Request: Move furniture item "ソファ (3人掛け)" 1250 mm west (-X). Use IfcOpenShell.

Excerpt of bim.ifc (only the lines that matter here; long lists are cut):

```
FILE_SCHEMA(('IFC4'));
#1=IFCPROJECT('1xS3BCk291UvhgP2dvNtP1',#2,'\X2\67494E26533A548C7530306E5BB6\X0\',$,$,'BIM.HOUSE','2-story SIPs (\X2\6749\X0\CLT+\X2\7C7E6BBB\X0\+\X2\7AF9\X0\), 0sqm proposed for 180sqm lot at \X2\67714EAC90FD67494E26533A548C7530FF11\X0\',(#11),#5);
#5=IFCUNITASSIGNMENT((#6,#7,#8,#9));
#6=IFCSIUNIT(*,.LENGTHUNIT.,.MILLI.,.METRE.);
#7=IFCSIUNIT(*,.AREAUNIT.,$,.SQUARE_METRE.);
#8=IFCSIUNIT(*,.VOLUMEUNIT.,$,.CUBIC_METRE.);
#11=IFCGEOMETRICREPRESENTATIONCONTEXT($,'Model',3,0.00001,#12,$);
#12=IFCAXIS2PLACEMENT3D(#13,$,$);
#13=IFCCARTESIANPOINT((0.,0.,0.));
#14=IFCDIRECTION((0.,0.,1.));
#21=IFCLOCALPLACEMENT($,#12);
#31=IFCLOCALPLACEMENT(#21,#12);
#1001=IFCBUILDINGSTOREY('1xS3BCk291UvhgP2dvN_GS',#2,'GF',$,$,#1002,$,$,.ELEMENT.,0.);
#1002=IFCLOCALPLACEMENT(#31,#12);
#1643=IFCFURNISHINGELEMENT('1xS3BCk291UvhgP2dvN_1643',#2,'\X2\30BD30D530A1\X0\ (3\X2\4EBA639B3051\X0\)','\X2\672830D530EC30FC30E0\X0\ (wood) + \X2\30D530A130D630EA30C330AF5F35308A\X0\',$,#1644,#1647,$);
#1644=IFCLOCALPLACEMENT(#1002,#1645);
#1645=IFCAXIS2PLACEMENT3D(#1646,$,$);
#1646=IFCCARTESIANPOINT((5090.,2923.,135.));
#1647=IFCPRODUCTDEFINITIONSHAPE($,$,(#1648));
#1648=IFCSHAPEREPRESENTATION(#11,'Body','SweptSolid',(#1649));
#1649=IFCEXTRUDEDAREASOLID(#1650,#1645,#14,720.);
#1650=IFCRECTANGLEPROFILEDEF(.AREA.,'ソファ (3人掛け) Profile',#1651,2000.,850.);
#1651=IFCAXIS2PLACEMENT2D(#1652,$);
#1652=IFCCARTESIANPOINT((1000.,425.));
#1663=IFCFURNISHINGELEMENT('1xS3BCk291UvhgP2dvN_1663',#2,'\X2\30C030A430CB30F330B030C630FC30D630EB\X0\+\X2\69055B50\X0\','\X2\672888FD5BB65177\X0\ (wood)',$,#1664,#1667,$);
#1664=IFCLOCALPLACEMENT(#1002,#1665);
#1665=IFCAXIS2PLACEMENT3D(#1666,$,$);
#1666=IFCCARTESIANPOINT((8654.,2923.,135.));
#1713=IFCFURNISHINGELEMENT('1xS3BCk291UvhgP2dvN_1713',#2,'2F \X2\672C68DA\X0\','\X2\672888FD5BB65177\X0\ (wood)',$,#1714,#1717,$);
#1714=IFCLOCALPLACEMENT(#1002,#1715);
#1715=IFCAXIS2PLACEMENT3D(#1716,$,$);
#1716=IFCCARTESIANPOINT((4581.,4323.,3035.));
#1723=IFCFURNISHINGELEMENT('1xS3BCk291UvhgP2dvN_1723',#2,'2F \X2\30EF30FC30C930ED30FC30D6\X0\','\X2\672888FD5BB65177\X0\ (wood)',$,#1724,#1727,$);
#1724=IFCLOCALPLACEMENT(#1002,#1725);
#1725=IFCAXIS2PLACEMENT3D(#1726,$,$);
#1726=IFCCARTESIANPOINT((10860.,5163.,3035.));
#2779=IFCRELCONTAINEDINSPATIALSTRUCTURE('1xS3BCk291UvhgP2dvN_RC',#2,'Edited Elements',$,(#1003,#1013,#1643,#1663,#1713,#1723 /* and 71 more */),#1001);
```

```python
import ifcopenshell
import ifcopenshell.api.geometry
import ifcopenshell.util.placement

model = ifcopenshell.open("bim.ifc")

item = model.by_id(1643)
matrix = ifcopenshell.util.placement.get_local_placement(item.ObjectPlacement)
matrix[0, 3] -= 1250.0
ifcopenshell.api.geometry.edit_object_placement(model, product=item, matrix=matrix, is_si=False)

print(ifcopenshell.util.placement.get_local_placement(item.ObjectPlacement).round(3) + 0.0)

model.write("bim_rev.ifc")
```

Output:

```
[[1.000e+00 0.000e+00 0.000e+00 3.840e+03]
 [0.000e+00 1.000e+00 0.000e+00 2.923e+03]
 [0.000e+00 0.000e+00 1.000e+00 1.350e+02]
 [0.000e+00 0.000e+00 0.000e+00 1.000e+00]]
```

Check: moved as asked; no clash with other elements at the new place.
